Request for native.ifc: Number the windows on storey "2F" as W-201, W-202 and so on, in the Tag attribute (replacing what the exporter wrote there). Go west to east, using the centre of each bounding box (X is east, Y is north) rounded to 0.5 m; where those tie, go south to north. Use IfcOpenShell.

First a look at what the model holds.

```python
import ifcopenshell
import ifcopenshell.util.element
import ifcopenshell.util.placement

model = ifcopenshell.open("native.ifc")
print(model.schema)
storey = next(s for s in model.by_type("IfcBuildingStorey") if s.Name == "2F")
windows = [e for e in ifcopenshell.util.element.get_decomposition(storey) if e.is_a("IfcWindow")]
for e in sorted(windows, key=lambda e: e.id()):
    origin = ifcopenshell.util.placement.get_local_placement(e.ObjectPlacement)[:3, 3]
    print(e.id(), e.Tag, e.Name, origin.round(2) + 0.0, sep=" | ")
```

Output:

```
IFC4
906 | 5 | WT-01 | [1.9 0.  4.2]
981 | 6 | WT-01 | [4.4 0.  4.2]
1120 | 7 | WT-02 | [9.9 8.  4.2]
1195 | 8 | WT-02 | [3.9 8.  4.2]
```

```python
import ifcopenshell
import ifcopenshell.geom
import ifcopenshell.util.element
import ifcopenshell.util.shape

model = ifcopenshell.open("native.ifc")
settings = ifcopenshell.geom.settings()
settings.set("use-world-coords", True)


def centre(element):
    shape = ifcopenshell.geom.create_shape(settings, element)
    return ifcopenshell.util.shape.get_bbox_centroid(shape.geometry)


storey = next(s for s in model.by_type("IfcBuildingStorey") if s.Name == "2F")
windows = [e for e in ifcopenshell.util.element.get_decomposition(storey) if e.is_a("IfcWindow")]

# Insertion points can sit at a corner or the storey origin, so sort by the geometry (in metres).
centres = {e: centre(e) for e in windows}
windows.sort(key=lambda e: (round(centres[e][0] / 0.5), centres[e][1]))

for i, e in enumerate(windows, start=1):
    number = f"W-2{i:02d}"
    e.Tag = number
    print(e.id(), number)

model.write("native_edited.ifc")
```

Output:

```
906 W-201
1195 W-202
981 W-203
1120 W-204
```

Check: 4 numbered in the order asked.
